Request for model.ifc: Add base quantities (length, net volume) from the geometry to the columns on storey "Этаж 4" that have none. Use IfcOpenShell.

First a look at what the model holds.

```python
import ifcopenshell
import ifcopenshell.util.element
import ifcopenshell.util.unit

model = ifcopenshell.open("model.ifc")
print(model.schema)
for unit_type in ("LENGTHUNIT", "AREAUNIT", "VOLUMEUNIT"):
    print(unit_type, ifcopenshell.util.unit.calculate_unit_scale(model, unit_type))
storey = next(s for s in model.by_type("IfcBuildingStorey") if s.Name == "Этаж 4")
columns = [e for e in ifcopenshell.util.element.get_decomposition(storey) if e.is_a("IfcColumn")]
for e in sorted(columns, key=lambda e: e.id()):
    print(e.id(), e.is_a(), e.Name, list(ifcopenshell.util.element.get_psets(e, qtos_only=True)), sep=" | ")
```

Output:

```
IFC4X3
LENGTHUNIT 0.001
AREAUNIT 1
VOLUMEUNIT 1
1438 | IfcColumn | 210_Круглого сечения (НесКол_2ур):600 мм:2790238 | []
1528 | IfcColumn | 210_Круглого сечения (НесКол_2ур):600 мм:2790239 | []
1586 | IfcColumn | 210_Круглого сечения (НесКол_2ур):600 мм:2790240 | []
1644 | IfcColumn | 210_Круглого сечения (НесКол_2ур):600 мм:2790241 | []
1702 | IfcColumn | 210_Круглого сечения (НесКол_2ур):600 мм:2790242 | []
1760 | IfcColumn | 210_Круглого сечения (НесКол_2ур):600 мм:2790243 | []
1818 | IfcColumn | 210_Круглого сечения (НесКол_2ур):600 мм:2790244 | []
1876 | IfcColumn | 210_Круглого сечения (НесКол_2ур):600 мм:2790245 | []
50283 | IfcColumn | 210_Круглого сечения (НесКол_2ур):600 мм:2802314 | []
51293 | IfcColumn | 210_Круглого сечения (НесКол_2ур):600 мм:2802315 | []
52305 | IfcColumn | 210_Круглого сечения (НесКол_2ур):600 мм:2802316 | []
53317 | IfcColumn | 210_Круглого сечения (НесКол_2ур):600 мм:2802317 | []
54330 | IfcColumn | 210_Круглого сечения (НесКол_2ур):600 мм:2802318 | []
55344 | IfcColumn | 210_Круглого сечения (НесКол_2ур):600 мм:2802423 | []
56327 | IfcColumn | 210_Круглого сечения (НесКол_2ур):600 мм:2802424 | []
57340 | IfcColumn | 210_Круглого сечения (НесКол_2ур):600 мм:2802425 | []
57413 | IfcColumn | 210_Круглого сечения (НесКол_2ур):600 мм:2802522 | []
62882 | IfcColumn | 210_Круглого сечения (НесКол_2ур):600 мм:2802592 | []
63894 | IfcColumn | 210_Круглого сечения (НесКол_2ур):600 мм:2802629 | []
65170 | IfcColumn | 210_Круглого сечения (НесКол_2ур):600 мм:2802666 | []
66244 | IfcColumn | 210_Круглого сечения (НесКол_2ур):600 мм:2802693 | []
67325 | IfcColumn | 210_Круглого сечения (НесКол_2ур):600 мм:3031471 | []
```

```python
import ifcopenshell
import ifcopenshell.api.pset
import ifcopenshell.geom
import ifcopenshell.util.element
import ifcopenshell.util.shape
import ifcopenshell.util.unit

model = ifcopenshell.open("model.ifc")
unit_scale = ifcopenshell.util.unit.calculate_unit_scale(model)
volume_scale = ifcopenshell.util.unit.calculate_unit_scale(model, "VOLUMEUNIT")
settings = ifcopenshell.geom.settings()

storey = next(s for s in model.by_type("IfcBuildingStorey") if s.Name == "Этаж 4")
columns = [e for e in ifcopenshell.util.element.get_decomposition(storey) if e.is_a("IfcColumn")]

for e in sorted(columns, key=lambda e: e.id()):
    if ifcopenshell.util.element.get_psets(e, qtos_only=True, should_inherit=False):
        continue
    # Geometry comes back in metres, in the element's own axes.
    shape = ifcopenshell.geom.create_shape(settings, e)
    values = {
        "Length": ifcopenshell.util.shape.get_z(shape.geometry) / unit_scale,
        "NetVolume": ifcopenshell.util.shape.get_volume(shape.geometry) / volume_scale,
    }
    qto = ifcopenshell.api.pset.add_qto(model, product=e, name="Qto_ColumnBaseQuantities")
    ifcopenshell.api.pset.edit_qto(model, qto=qto, properties=values)
    print(e.id(), {k: round(v, 3) for k, v in values.items()})

model.write("model_v2.ifc")
```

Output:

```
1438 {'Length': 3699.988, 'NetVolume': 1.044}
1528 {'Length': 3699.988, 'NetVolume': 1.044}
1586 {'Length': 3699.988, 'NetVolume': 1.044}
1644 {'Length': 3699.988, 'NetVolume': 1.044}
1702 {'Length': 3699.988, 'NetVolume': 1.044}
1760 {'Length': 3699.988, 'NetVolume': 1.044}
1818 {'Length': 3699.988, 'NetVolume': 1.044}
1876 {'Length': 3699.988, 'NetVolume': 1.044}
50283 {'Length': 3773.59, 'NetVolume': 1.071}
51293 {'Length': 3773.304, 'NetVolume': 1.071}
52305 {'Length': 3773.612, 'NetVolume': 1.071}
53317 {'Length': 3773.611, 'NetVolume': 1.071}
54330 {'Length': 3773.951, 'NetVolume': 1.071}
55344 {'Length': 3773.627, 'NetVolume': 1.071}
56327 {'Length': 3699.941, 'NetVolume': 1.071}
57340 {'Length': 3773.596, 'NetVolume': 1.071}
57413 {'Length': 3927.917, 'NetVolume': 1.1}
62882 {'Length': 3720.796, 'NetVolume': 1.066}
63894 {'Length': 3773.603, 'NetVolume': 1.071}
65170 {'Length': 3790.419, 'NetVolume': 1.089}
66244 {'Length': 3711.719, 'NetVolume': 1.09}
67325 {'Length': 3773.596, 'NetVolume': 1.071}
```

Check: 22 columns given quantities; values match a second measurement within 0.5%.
